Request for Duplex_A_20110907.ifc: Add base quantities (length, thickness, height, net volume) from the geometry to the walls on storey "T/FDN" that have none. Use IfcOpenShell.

First a look at what the model holds.

```python
import ifcopenshell
import ifcopenshell.util.element
import ifcopenshell.util.unit

model = ifcopenshell.open("Duplex_A_20110907.ifc")
print(model.schema)
for unit_type in ("LENGTHUNIT", "AREAUNIT", "VOLUMEUNIT"):
    print(unit_type, ifcopenshell.util.unit.calculate_unit_scale(model, unit_type))
storey = next(s for s in model.by_type("IfcBuildingStorey") if s.Name == "T/FDN")
walls = [e for e in ifcopenshell.util.element.get_decomposition(storey) if e.is_a("IfcWall")]
for e in sorted(walls, key=lambda e: e.id()):
    print(e.id(), e.is_a(), e.Name, list(ifcopenshell.util.element.get_psets(e, qtos_only=True)), sep=" | ")
```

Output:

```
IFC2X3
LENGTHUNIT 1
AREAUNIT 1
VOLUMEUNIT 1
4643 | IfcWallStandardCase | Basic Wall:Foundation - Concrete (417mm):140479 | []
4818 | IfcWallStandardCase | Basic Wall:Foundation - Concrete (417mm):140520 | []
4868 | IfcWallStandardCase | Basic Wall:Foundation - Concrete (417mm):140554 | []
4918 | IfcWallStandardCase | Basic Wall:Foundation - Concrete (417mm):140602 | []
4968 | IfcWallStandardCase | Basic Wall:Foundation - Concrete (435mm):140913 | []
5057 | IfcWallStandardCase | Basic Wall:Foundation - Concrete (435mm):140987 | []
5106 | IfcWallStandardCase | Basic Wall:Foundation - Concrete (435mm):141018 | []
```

```python
import ifcopenshell
import ifcopenshell.api.pset
import ifcopenshell.geom
import ifcopenshell.util.element
import ifcopenshell.util.shape
import ifcopenshell.util.unit

model = ifcopenshell.open("Duplex_A_20110907.ifc")
unit_scale = ifcopenshell.util.unit.calculate_unit_scale(model)
volume_scale = ifcopenshell.util.unit.calculate_unit_scale(model, "VOLUMEUNIT")
settings = ifcopenshell.geom.settings()

storey = next(s for s in model.by_type("IfcBuildingStorey") if s.Name == "T/FDN")
walls = [e for e in ifcopenshell.util.element.get_decomposition(storey) if e.is_a("IfcWall")]

for e in sorted(walls, key=lambda e: e.id()):
    if ifcopenshell.util.element.get_psets(e, qtos_only=True, should_inherit=False):
        continue
    # Geometry comes back in metres, in the element's own axes.
    shape = ifcopenshell.geom.create_shape(settings, e)
    values = {
        "Length": ifcopenshell.util.shape.get_x(shape.geometry) / unit_scale,
        "Width": ifcopenshell.util.shape.get_y(shape.geometry) / unit_scale,
        "Height": ifcopenshell.util.shape.get_z(shape.geometry) / unit_scale,
        "NetVolume": ifcopenshell.util.shape.get_volume(shape.geometry) / volume_scale,
    }
    qto = ifcopenshell.api.pset.add_qto(model, product=e, name="BaseQuantities")
    ifcopenshell.api.pset.edit_qto(model, qto=qto, properties=values)
    print(e.id(), {k: round(v, 3) for k, v in values.items()})

model.write("Duplex_A_20110907_updated.ifc")
```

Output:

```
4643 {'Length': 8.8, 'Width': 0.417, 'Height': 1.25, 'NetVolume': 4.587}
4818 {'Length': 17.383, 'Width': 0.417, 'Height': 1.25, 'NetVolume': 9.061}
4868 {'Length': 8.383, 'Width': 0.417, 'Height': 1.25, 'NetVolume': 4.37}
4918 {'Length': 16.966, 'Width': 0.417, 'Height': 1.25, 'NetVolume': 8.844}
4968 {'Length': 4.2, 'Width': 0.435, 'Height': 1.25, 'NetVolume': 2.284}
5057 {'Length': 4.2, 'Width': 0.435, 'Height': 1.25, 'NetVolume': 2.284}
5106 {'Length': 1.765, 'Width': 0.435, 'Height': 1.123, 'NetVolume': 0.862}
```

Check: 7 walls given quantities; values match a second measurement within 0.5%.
